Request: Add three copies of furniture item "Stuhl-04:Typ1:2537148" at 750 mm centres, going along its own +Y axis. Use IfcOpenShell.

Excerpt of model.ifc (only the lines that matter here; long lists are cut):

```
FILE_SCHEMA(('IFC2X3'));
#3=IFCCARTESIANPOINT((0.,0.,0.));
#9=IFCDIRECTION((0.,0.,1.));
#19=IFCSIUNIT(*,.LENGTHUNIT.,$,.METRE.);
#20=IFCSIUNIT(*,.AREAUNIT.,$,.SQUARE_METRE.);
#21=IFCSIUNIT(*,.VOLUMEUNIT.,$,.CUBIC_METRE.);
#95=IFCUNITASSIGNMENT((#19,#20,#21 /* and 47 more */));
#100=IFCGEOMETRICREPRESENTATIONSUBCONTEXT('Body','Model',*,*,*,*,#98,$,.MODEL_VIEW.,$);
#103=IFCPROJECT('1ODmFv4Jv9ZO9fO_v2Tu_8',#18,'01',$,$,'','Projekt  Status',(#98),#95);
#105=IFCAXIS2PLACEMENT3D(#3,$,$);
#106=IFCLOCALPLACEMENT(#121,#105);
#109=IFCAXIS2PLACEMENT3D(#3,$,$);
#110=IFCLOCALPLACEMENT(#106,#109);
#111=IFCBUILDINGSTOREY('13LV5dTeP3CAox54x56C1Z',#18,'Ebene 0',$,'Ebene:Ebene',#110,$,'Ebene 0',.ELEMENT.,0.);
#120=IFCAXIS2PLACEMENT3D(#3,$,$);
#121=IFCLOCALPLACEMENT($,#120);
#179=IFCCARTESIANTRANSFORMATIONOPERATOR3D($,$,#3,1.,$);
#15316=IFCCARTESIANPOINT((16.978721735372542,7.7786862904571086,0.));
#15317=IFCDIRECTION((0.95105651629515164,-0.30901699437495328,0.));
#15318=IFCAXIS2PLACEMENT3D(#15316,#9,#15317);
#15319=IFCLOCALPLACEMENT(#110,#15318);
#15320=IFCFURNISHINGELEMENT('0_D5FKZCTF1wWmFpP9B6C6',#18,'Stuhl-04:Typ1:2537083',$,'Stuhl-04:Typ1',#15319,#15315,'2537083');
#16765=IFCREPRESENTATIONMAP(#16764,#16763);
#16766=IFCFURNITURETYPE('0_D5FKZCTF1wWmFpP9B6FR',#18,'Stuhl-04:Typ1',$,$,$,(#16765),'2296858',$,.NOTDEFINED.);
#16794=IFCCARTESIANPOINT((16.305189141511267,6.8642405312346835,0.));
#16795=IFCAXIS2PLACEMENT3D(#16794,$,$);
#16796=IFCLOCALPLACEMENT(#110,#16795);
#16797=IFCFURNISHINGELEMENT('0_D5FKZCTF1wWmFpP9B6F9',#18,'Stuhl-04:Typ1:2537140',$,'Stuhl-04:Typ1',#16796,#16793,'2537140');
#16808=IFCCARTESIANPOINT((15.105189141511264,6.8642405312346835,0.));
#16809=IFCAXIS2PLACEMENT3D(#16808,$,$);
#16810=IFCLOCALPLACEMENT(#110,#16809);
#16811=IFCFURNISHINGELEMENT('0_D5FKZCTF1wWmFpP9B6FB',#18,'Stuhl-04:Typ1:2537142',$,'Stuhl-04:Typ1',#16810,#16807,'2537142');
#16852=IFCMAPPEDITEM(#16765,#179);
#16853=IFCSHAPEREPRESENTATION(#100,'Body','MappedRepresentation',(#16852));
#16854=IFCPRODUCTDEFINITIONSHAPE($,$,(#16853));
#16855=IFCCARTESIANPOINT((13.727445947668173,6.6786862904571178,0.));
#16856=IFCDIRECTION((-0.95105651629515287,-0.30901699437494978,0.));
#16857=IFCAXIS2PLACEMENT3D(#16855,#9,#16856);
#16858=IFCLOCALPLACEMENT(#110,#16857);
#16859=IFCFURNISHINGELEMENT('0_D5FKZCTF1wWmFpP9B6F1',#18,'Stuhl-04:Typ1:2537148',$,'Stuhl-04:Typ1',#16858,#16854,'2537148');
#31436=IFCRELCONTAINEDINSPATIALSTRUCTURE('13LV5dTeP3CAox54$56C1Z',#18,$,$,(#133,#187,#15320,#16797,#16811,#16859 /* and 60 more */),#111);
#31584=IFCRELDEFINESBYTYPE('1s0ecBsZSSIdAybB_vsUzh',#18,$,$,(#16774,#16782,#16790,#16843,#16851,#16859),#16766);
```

```python
import ifcopenshell
import ifcopenshell.api.geometry
import ifcopenshell.api.root
import ifcopenshell.util.element
import ifcopenshell.util.placement
import ifcopenshell.util.unit

model = ifcopenshell.open("model.ifc")
unit_scale = ifcopenshell.util.unit.calculate_unit_scale(model)

source = model.by_guid("0_D5FKZCTF1wWmFpP9B6F1")
base = ifcopenshell.util.placement.get_local_placement(source.ObjectPlacement)
step = base[:3, 1] * 0.75 / unit_scale

for i in range(1, 4):
    copy = ifcopenshell.api.root.copy_class(model, product=source)
    copy.Representation = ifcopenshell.util.element.copy_deep(
        model, source.Representation, exclude=["IfcGeometricRepresentationContext", "IfcRepresentationMap"]
    )
    copy.Name = "Stuhl-04:Typ1"
    copy.Tag = None
    matrix = base.copy()
    matrix[:3, 3] += i * step
    print("added at", matrix[:3, 3].round(3) + 0.0)
    ifcopenshell.api.geometry.edit_object_placement(model, product=copy, matrix=matrix, is_si=False)

model.write("model_v2.ifc")
```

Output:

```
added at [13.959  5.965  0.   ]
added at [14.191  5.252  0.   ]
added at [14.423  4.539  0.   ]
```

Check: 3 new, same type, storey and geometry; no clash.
